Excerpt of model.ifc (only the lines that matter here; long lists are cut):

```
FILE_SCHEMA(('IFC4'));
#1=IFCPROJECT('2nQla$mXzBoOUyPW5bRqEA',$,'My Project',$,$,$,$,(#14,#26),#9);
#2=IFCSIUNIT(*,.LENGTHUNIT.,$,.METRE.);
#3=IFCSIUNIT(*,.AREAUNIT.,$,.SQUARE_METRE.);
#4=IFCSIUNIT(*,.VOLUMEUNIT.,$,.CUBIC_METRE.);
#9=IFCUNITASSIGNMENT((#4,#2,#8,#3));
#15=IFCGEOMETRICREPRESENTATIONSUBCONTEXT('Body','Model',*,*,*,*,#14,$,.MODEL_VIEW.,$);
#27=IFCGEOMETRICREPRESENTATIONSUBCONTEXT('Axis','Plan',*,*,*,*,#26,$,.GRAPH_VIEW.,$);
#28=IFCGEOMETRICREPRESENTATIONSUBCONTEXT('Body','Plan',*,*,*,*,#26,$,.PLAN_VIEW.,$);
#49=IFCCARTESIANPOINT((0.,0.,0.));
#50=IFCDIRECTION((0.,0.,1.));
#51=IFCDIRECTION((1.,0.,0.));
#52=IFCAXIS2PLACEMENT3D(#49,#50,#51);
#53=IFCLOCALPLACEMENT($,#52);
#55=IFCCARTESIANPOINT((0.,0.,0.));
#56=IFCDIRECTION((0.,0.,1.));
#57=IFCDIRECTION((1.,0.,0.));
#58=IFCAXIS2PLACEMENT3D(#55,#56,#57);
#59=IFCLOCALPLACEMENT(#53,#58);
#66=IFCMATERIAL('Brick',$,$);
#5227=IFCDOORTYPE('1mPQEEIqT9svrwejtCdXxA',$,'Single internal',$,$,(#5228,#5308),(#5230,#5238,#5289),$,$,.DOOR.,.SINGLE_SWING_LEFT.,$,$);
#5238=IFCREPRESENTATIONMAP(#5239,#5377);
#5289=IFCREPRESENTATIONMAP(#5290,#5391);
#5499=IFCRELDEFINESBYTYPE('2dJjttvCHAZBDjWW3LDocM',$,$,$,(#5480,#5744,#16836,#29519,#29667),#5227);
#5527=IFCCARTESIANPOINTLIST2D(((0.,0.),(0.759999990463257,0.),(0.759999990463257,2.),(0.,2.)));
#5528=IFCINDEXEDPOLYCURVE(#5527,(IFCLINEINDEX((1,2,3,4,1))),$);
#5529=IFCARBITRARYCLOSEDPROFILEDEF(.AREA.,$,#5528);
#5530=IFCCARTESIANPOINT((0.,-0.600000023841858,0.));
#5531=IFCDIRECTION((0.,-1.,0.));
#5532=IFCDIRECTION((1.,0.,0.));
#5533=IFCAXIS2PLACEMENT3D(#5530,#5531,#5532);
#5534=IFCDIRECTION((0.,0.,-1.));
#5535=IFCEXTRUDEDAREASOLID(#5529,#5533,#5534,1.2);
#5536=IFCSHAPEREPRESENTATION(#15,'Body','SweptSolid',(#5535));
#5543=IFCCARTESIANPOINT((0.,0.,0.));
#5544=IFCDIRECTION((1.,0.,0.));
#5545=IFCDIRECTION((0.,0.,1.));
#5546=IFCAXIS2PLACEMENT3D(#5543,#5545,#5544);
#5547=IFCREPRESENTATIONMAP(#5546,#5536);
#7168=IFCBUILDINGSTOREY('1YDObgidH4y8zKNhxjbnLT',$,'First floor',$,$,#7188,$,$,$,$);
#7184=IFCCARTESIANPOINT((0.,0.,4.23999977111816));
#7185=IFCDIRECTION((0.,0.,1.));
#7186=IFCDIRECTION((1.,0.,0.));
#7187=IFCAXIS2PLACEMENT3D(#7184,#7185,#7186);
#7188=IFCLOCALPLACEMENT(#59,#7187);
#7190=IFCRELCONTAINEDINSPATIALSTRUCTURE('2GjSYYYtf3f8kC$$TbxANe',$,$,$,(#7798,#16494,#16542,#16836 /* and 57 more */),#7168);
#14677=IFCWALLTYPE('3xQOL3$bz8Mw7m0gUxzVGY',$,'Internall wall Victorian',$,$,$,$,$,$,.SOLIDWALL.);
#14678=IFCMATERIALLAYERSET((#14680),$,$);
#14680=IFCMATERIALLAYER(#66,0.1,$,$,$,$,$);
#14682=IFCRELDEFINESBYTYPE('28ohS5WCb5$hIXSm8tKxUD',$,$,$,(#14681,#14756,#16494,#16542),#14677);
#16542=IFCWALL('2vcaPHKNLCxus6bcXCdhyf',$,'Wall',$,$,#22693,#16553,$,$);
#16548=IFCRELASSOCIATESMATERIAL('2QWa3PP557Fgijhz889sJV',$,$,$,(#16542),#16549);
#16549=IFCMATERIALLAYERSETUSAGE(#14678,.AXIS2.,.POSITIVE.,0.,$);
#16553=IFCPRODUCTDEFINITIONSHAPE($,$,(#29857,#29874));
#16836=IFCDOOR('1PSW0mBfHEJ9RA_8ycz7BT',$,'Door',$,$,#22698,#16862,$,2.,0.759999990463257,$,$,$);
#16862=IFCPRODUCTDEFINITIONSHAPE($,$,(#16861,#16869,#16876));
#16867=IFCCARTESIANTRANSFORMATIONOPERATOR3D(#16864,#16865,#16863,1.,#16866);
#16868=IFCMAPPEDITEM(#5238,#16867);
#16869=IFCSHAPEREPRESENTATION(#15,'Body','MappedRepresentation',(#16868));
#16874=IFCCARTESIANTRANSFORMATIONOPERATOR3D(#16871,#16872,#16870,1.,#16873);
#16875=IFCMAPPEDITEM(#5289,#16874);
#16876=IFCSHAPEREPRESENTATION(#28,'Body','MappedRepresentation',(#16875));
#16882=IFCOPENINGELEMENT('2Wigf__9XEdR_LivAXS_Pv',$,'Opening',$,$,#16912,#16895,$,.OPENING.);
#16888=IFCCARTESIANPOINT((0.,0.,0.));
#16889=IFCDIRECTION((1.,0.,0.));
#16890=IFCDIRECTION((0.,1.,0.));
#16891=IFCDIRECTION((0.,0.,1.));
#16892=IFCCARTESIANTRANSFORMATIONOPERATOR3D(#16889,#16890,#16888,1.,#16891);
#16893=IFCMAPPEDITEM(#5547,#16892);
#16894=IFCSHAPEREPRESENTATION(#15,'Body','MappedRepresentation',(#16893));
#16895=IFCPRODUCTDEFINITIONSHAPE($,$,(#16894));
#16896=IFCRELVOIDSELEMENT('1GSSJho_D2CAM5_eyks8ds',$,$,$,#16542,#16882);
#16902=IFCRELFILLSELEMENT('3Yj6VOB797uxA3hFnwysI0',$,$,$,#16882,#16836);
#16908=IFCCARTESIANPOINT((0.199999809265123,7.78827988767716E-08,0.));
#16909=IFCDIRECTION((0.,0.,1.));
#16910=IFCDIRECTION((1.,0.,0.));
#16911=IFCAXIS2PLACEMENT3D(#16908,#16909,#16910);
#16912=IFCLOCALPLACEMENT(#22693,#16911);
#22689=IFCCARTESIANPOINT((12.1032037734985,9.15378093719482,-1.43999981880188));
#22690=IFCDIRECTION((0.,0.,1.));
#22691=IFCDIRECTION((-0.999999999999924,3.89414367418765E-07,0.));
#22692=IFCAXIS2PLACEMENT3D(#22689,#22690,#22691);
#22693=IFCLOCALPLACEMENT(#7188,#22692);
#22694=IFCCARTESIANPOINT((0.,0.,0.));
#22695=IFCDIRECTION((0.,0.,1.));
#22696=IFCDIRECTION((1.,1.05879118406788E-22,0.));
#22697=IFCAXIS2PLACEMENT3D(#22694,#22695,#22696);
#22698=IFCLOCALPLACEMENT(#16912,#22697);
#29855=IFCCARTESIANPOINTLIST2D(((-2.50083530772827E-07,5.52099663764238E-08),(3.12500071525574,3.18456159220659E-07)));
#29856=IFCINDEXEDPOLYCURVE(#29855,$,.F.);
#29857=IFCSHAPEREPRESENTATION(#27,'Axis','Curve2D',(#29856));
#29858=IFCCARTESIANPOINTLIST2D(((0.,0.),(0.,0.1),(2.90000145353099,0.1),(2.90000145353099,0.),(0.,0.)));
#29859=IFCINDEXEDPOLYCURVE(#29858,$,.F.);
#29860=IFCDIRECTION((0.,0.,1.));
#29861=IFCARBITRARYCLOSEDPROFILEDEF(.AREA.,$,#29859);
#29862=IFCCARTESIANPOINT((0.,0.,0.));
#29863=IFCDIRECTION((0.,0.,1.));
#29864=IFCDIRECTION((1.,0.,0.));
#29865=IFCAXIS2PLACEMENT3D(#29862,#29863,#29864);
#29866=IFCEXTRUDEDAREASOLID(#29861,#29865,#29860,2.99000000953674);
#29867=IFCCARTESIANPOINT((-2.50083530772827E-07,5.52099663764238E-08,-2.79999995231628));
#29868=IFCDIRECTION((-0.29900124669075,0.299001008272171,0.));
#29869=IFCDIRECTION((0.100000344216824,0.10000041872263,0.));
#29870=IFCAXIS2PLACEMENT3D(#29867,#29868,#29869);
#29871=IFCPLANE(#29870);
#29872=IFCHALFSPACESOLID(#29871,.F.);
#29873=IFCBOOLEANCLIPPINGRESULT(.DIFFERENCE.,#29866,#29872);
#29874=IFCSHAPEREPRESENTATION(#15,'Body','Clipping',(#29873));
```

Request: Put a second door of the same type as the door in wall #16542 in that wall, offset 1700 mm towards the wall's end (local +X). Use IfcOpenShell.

```python
import ifcopenshell
import ifcopenshell.api.feature
import ifcopenshell.api.geometry
import ifcopenshell.api.root
import ifcopenshell.geom
import ifcopenshell.util.element
import ifcopenshell.util.placement
import ifcopenshell.util.shape

model = ifcopenshell.open("model.ifc")
settings = ifcopenshell.geom.settings()


def volume(element):
    """Net volume in cubic metres, openings subtracted."""
    shape = ifcopenshell.geom.create_shape(settings, element)
    return ifcopenshell.util.shape.get_volume(shape.geometry)


door = model.by_guid("1PSW0mBfHEJ9RA_8ycz7BT")
opening = door.FillsVoids[0].RelatingOpeningElement
wall = opening.VoidsElements[0].RelatingBuildingElement
before = volume(wall)
shift = ifcopenshell.util.placement.get_local_placement(wall.ObjectPlacement)[:3, 0] * 1.7

# copy_class copies the void relationship, type, container and properties, but no geometry.
new_opening = ifcopenshell.api.root.copy_class(model, product=opening)
new_opening.Representation = ifcopenshell.util.element.copy_deep(
    model, opening.Representation, exclude=["IfcGeometricRepresentationContext", "IfcRepresentationMap"]
)
new_door = ifcopenshell.api.root.copy_class(model, product=door)
new_door.Representation = ifcopenshell.util.element.copy_deep(
    model, door.Representation, exclude=["IfcGeometricRepresentationContext", "IfcRepresentationMap"]
)
ifcopenshell.api.feature.add_filling(model, opening=new_opening, element=new_door)

for old, new in ((opening, new_opening), (door, new_door)):
    matrix = ifcopenshell.util.placement.get_local_placement(old.ObjectPlacement)
    matrix[:3, 3] += shift
    ifcopenshell.api.geometry.edit_object_placement(model, product=new, matrix=matrix, is_si=False)

after = volume(wall)

print(f"wall volume {before:.3f} -> {after:.3f} m3")

model.write("model_edited.ifc")
```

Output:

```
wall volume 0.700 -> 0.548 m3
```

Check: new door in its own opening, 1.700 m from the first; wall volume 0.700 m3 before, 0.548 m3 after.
